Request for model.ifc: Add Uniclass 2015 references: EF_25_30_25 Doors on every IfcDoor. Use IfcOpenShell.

First a look at what the model holds.

```python
import ifcopenshell

model = ifcopenshell.open("model.ifc")
print(model.schema)
print("classifications:", [c.Name for c in model.by_type("IfcClassification")])
for ifc_class in ("IfcDoor", "IfcRoof", "IfcStair", "IfcWall", "IfcWindow"):
    print(ifc_class, len(model.by_type(ifc_class)))
```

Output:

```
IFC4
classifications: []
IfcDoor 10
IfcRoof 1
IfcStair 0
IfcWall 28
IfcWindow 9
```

```python
import ifcopenshell
import ifcopenshell.api.classification

model = ifcopenshell.open("model.ifc")

system = ifcopenshell.api.classification.add_classification(model, classification="Uniclass 2015")

codes = {
    "IfcDoor": ("EF_25_30_25", "Doors"),
}
for ifc_class, (code, name) in codes.items():
    products = model.by_type(ifc_class)
    ifcopenshell.api.classification.add_reference(
        model, products=products, classification=system, identification=code, name=name
    )
    print(code, len(products))

model.write("model_edited.ifc")
```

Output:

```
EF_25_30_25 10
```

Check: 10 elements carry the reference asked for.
